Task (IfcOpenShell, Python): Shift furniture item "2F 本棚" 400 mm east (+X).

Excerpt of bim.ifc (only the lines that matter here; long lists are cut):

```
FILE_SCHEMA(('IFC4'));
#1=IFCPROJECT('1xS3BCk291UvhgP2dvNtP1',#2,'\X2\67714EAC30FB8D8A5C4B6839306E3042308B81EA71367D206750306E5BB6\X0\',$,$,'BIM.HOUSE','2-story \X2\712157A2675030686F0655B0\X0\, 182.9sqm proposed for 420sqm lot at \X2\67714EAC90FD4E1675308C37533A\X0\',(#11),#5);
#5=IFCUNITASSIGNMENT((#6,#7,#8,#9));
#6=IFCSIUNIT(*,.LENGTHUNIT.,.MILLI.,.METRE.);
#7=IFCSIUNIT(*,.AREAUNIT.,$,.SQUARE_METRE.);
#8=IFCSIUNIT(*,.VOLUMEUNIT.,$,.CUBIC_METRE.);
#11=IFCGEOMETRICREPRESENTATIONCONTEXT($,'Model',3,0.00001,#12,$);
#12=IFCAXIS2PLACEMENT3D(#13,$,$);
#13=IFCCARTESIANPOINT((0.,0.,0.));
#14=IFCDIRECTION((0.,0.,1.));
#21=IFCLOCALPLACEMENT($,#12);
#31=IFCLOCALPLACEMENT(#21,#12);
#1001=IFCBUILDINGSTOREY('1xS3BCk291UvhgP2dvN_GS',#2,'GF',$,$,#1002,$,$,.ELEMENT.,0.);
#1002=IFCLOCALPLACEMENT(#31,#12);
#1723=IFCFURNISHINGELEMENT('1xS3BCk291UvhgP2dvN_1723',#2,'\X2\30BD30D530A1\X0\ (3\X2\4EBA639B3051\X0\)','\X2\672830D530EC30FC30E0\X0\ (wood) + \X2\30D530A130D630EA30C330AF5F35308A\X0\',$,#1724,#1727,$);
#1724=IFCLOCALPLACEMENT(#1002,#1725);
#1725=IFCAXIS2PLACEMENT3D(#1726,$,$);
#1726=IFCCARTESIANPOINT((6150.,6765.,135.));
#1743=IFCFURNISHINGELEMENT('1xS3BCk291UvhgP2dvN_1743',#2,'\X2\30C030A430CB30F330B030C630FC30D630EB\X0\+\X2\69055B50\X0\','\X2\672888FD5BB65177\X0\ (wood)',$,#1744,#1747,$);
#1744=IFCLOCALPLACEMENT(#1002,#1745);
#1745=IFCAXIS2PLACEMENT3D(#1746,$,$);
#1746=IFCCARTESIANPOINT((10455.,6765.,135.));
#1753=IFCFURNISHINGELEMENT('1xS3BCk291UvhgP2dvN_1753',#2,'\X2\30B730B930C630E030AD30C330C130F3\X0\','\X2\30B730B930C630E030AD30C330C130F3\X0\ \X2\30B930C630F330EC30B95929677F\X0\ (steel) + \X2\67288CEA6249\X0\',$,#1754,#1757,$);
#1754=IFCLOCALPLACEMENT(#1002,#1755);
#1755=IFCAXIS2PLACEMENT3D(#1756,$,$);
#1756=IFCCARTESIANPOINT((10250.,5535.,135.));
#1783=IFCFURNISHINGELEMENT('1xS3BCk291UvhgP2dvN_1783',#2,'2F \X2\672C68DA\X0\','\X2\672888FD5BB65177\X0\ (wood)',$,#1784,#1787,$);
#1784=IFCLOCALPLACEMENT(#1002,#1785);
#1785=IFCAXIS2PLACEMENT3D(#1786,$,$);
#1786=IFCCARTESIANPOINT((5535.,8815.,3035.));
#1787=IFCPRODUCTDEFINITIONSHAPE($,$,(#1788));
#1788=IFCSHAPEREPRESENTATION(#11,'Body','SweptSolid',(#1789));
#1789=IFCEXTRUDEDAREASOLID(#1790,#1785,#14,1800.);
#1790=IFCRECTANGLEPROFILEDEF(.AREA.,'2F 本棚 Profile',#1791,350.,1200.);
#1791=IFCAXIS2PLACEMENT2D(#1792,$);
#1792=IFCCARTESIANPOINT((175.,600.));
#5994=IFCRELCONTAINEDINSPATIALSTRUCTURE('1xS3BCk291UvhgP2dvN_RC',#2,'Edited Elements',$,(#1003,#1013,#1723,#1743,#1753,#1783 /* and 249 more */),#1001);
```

```python
import ifcopenshell
import ifcopenshell.api.geometry
import ifcopenshell.util.placement
import ifcopenshell.util.unit

model = ifcopenshell.open("bim.ifc")
unit_scale = ifcopenshell.util.unit.calculate_unit_scale(model)

item = model.by_guid("1xS3BCk291UvhgP2dvN_1783")
matrix = ifcopenshell.util.placement.get_local_placement(item.ObjectPlacement)
matrix[0, 3] += 0.4 / unit_scale
ifcopenshell.api.geometry.edit_object_placement(model, product=item, matrix=matrix, is_si=False)

print(ifcopenshell.util.placement.get_local_placement(item.ObjectPlacement).round(3) + 0.0)

model.write("bim_rev.ifc")
```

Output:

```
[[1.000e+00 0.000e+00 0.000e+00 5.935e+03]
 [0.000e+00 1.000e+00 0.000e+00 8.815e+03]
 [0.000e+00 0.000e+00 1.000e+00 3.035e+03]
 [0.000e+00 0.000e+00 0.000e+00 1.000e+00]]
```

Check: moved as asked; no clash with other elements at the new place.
